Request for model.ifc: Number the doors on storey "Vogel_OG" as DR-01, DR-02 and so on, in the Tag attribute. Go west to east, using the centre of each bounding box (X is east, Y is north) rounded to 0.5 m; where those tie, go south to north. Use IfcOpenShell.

First a look at what the model holds.

```python
import ifcopenshell
import ifcopenshell.util.element
import ifcopenshell.util.placement

model = ifcopenshell.open("model.ifc")
print(model.schema)
storey = next(s for s in model.by_type("IfcBuildingStorey") if s.Name == "Vogel_OG")
doors = [e for e in ifcopenshell.util.element.get_decomposition(storey) if e.is_a("IfcDoor")]
for e in sorted(doors, key=lambda e: e.id()):
    origin = ifcopenshell.util.placement.get_local_placement(e.ObjectPlacement)[:3, 3]
    print(e.id(), e.Tag, e.Name, origin.round(2) + 0.0, sep=" | ")
```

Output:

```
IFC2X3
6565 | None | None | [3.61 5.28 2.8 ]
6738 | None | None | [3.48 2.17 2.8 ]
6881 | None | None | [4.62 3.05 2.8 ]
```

```python
import ifcopenshell
import ifcopenshell.geom
import ifcopenshell.util.element
import ifcopenshell.util.shape

model = ifcopenshell.open("model.ifc")
settings = ifcopenshell.geom.settings()
settings.set("use-world-coords", True)


def centre(element):
    shape = ifcopenshell.geom.create_shape(settings, element)
    return ifcopenshell.util.shape.get_bbox_centroid(shape.geometry)


storey = next(s for s in model.by_type("IfcBuildingStorey") if s.Name == "Vogel_OG")
doors = [e for e in ifcopenshell.util.element.get_decomposition(storey) if e.is_a("IfcDoor")]

# Insertion points can sit at a corner or the storey origin, so sort by the geometry (in metres).
centres = {e: centre(e) for e in doors}
doors.sort(key=lambda e: (round(centres[e][0] / 0.5), centres[e][1]))

for i, e in enumerate(doors, start=1):
    number = f"DR-{i:02d}"
    e.Tag = number
    print(e.id(), number)

model.write("model_v2.ifc")
```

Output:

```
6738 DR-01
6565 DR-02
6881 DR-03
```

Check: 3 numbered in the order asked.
